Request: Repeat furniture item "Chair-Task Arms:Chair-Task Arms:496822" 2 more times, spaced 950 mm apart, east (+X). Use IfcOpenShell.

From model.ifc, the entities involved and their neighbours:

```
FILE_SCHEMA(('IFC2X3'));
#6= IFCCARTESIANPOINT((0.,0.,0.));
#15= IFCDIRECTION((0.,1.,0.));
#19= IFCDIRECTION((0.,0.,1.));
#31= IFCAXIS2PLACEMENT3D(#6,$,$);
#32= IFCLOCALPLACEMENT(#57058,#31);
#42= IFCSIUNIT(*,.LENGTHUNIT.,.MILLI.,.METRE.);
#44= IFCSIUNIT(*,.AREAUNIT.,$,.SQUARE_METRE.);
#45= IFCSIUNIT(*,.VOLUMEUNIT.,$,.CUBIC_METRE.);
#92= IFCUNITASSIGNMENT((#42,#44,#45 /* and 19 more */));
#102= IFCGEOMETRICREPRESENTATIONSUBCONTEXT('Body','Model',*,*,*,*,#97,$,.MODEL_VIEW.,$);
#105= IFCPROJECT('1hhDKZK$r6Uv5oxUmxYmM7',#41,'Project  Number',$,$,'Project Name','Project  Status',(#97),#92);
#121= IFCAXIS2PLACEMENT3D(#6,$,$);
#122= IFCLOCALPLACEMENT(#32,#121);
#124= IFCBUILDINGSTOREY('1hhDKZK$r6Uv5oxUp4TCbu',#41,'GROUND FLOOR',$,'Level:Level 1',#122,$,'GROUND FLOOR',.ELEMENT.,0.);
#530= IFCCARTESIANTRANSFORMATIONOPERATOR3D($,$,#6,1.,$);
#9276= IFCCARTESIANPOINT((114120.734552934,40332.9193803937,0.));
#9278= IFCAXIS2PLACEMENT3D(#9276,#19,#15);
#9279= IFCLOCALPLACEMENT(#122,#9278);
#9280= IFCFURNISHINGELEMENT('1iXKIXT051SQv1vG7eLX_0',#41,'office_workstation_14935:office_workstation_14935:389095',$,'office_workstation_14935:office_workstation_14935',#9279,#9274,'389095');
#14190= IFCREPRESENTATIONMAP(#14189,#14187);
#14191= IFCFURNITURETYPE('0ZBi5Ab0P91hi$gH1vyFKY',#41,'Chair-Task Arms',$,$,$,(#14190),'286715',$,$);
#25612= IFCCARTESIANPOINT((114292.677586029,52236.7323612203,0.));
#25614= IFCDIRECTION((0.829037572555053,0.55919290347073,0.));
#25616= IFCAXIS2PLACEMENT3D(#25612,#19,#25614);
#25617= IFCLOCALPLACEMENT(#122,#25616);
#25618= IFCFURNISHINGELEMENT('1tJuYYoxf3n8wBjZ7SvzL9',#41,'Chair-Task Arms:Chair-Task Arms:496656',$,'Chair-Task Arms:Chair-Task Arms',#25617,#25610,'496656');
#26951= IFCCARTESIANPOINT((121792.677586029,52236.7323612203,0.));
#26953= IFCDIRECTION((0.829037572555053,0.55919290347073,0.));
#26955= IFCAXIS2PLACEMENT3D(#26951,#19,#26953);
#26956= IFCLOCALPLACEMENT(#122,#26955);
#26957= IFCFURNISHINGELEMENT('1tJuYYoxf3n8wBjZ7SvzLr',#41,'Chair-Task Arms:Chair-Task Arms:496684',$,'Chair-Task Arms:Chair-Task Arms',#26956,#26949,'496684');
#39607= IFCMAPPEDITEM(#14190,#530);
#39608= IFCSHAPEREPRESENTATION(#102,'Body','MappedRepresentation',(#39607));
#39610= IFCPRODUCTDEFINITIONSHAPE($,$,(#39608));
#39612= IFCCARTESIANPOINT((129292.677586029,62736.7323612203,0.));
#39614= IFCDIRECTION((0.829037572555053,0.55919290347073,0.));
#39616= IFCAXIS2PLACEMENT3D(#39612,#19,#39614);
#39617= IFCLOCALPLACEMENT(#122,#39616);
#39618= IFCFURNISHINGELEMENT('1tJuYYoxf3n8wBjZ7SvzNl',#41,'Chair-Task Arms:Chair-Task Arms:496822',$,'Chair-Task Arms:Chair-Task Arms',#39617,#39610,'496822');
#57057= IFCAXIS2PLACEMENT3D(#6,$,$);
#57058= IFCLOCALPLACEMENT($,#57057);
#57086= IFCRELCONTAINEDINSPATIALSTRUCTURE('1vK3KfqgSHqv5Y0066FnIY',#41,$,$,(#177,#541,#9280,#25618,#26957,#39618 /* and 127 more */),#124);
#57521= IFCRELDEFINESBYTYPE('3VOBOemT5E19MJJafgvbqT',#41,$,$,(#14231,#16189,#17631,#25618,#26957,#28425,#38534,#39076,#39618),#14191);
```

```python
import numpy as np
import ifcopenshell
import ifcopenshell.api.geometry
import ifcopenshell.api.root
import ifcopenshell.util.element
import ifcopenshell.util.placement
import ifcopenshell.util.unit

model = ifcopenshell.open("model.ifc")
unit_scale = ifcopenshell.util.unit.calculate_unit_scale(model)


def reuse_history(source, copy):
    """copy_class also copies each property set's owner history, people and application; keep the originals."""
    for rel in copy.IsDefinedBy:
        if rel.is_a("IfcRelDefinesByProperties") and (history := rel.RelatingPropertyDefinition.OwnerHistory):
            rel.RelatingPropertyDefinition.OwnerHistory = source.OwnerHistory
            ifcopenshell.util.element.remove_deep2(model, history)


source = model.by_guid("1tJuYYoxf3n8wBjZ7SvzNl")
base = ifcopenshell.util.placement.get_local_placement(source.ObjectPlacement)
step = np.array([1.0, 0.0, 0.0]) * 0.95 / unit_scale

for i in range(1, 3):
    copy = ifcopenshell.api.root.copy_class(model, product=source)
    copy.Representation = ifcopenshell.util.element.copy_deep(
        model, source.Representation, exclude=["IfcGeometricRepresentationContext", "IfcRepresentationMap"]
    )
    copy.Name = "Chair-Task Arms:Chair-Task Arms"
    copy.Tag = None
    reuse_history(source, copy)
    matrix = base.copy()
    matrix[:3, 3] += i * step
    print("added at", matrix[:3, 3].round(3) + 0.0)
    ifcopenshell.api.geometry.edit_object_placement(model, product=copy, matrix=matrix, is_si=False)

model.write("model_rev.ifc")
```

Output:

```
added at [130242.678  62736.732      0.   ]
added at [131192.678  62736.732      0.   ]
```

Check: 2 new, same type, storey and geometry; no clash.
